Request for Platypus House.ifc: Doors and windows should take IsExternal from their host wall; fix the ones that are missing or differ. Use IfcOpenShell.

First a look at what the model holds.

```python
import ifcopenshell
import ifcopenshell.util.element

model = ifcopenshell.open("Platypus House.ifc")
print(model.schema)
seen = {}
for e in model.by_type("IfcDoor") + model.by_type("IfcWindow"):
    if not e.FillsVoids:
        continue
    host = e.FillsVoids[0].RelatingOpeningElement.VoidsElements[0].RelatingBuildingElement
    own = ifcopenshell.util.element.get_pset(e, f"Pset_{e.is_a()[3:].removesuffix('StandardCase')}Common", "IsExternal")
    wall = ifcopenshell.util.element.get_pset(host, "Pset_WallCommon", "IsExternal")
    seen[e.is_a(), own, wall] = seen.get((e.is_a(), own, wall), 0) + 1
for (cls, own, wall), count in sorted(seen.items(), key=str):
    print(count, cls, "IsExternal:", own, "| host wall:", wall)
```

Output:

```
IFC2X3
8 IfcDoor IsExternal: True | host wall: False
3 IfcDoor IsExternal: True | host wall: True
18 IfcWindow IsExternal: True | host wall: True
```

```python
import ifcopenshell
import ifcopenshell.api.pset
import ifcopenshell.util.element

model = ifcopenshell.open("Platypus House.ifc")

count = 0
for ifc_class, pset_name in (("IfcDoor", "Pset_DoorCommon"), ("IfcWindow", "Pset_WindowCommon")):
    for e in model.by_type(ifc_class):
        if not e.FillsVoids:
            continue
        host = e.FillsVoids[0].RelatingOpeningElement.VoidsElements[0].RelatingBuildingElement
        external = ifcopenshell.util.element.get_pset(host, "Pset_WallCommon", "IsExternal")
        if external is None or ifcopenshell.util.element.get_pset(e, pset_name, "IsExternal") == external:
            continue
        pset = ifcopenshell.api.pset.add_pset(model, product=e, name=pset_name)
        ifcopenshell.api.pset.edit_pset(model, pset=pset, properties={"IsExternal": external})
        count += 1

print(count, "updated")

model.write("Platypus House_rev.ifc")
```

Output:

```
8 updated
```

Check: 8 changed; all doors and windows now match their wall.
